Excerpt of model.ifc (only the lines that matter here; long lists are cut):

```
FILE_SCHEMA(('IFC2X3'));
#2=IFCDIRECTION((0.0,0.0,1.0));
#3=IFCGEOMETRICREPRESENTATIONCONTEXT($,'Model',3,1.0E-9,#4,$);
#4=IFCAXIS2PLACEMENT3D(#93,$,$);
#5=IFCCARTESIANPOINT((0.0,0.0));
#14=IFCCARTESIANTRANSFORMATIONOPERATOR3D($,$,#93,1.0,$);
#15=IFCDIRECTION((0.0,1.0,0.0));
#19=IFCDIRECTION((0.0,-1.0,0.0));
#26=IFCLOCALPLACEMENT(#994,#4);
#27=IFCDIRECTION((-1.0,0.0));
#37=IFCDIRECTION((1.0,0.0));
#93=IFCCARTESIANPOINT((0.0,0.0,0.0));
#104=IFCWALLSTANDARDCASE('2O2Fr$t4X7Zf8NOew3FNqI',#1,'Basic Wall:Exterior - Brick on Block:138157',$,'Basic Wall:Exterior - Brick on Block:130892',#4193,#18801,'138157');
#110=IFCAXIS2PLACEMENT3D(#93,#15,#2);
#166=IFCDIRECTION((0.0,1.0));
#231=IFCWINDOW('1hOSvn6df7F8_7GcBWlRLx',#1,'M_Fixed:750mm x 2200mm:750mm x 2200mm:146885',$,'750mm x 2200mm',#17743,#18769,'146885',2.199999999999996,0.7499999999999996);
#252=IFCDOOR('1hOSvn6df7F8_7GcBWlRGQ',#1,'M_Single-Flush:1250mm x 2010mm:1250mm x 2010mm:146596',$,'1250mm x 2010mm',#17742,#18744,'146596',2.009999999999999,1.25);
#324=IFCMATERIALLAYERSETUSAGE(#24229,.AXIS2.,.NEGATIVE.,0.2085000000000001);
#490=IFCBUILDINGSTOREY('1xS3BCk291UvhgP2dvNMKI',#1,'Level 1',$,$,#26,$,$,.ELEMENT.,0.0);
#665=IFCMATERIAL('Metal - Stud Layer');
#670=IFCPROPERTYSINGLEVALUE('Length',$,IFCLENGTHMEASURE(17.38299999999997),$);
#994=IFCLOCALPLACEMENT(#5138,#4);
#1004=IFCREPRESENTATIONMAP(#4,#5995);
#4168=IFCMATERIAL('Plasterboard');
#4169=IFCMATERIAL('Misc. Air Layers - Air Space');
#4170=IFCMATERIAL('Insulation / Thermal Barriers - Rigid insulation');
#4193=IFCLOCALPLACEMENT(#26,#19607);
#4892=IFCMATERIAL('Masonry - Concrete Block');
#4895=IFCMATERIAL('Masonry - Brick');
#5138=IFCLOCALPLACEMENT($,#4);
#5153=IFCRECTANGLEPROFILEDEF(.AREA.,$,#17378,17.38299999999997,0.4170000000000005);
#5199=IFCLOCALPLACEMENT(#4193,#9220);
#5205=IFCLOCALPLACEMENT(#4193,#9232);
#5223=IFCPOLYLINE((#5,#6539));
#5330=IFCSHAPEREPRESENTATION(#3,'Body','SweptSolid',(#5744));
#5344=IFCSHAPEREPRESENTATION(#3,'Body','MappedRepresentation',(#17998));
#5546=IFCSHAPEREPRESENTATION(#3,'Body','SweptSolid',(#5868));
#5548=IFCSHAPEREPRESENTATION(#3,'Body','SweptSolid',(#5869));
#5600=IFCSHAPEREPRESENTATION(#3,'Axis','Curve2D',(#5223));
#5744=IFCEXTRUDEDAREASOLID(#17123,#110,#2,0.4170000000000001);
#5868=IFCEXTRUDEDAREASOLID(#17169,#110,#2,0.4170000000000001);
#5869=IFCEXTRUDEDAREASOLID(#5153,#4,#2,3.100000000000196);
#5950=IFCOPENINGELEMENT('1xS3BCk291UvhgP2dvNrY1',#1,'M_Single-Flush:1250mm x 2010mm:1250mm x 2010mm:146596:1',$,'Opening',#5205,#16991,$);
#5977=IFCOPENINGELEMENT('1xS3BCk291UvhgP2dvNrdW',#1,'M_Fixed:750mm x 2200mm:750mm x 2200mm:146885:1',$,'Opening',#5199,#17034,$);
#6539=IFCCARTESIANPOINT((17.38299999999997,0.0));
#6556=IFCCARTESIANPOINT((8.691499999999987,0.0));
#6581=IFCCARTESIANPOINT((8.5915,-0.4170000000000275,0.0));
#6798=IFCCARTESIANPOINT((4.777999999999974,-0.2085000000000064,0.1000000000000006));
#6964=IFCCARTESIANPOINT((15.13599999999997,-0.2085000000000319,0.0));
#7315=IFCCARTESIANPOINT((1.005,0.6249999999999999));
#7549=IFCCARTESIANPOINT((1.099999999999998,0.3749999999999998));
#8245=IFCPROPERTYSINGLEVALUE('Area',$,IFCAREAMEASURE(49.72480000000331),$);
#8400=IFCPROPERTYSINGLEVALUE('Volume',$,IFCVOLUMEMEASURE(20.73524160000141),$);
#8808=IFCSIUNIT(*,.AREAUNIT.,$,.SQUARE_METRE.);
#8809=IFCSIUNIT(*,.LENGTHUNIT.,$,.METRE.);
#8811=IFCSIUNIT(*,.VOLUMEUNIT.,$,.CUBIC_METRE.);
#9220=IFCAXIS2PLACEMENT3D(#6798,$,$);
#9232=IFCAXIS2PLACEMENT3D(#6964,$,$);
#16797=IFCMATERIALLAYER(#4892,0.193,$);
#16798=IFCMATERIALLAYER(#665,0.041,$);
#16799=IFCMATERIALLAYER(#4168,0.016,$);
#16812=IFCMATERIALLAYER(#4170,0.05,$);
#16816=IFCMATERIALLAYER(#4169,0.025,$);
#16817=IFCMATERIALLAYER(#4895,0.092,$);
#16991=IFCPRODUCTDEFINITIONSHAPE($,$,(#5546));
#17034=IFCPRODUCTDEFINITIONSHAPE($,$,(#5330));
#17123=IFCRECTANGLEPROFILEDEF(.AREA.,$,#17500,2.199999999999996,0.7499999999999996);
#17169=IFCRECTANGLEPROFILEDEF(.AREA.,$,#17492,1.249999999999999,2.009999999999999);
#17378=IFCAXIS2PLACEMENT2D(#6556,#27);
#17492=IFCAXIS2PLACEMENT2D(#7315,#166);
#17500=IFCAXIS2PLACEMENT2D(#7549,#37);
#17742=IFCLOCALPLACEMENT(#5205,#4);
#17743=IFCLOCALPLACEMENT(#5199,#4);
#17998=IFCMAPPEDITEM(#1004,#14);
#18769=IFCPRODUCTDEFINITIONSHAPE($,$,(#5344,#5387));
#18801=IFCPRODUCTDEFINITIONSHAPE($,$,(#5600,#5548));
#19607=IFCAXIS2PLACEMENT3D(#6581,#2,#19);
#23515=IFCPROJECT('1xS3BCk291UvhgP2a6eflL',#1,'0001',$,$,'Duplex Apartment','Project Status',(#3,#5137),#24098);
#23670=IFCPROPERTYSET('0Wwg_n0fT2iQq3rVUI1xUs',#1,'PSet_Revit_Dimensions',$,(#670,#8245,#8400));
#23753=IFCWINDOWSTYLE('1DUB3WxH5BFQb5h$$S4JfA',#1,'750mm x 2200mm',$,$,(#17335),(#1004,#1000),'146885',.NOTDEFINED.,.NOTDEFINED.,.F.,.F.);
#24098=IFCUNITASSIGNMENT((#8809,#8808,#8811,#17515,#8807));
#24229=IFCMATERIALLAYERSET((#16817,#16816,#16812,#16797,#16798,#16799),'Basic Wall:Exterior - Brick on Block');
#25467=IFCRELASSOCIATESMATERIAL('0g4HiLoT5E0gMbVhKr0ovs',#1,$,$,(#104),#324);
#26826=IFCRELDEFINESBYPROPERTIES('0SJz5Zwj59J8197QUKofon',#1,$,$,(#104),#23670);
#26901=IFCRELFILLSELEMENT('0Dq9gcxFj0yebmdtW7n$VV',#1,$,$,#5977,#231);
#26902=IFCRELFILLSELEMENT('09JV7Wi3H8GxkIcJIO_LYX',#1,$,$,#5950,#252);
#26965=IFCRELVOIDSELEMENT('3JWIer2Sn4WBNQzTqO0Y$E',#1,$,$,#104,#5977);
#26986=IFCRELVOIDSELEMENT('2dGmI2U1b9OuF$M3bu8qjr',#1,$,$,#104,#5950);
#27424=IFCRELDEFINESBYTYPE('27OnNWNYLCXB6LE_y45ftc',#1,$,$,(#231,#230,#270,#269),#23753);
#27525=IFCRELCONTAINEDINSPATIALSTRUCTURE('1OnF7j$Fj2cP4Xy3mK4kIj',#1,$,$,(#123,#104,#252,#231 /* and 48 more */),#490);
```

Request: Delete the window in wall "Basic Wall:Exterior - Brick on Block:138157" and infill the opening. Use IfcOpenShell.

```python
import ifcopenshell
import ifcopenshell.api.feature
import ifcopenshell.api.pset
import ifcopenshell.api.root
import ifcopenshell.geom
import ifcopenshell.util.element
import ifcopenshell.util.shape
import ifcopenshell.util.unit

model = ifcopenshell.open("model.ifc")
area_scale = ifcopenshell.util.unit.calculate_unit_scale(model, "AREAUNIT")
volume_scale = ifcopenshell.util.unit.calculate_unit_scale(model, "VOLUMEUNIT")
settings = ifcopenshell.geom.settings()


def volume(element):
    """Net volume in cubic metres, openings subtracted."""
    shape = ifcopenshell.geom.create_shape(settings, element)
    return ifcopenshell.util.shape.get_volume(shape.geometry)


window = model.by_guid("1hOSvn6df7F8_7GcBWlRLx")
opening = window.FillsVoids[0].RelatingOpeningElement
wall = opening.VoidsElements[0].RelatingBuildingElement
before = volume(wall)

ifcopenshell.api.root.remove_product(model, product=window)
ifcopenshell.api.feature.remove_feature(model, feature=opening)

after = volume(wall)
thickness = 0.417  # wall thickness in metres

# Update the wall's stored quantities.
pset = model.by_id(ifcopenshell.util.element.get_pset(wall, "PSet_Revit_Dimensions", should_inherit=False)["id"])
ifcopenshell.api.pset.edit_pset(model, pset=pset, properties={
    "Area": model.create_entity("IfcAreaMeasure", after / thickness / area_scale),
    "Volume": model.create_entity("IfcVolumeMeasure", after / volume_scale),
})

print(f"wall volume {before:.3f} -> {after:.3f} m3")

model.write("model-out.ifc")
```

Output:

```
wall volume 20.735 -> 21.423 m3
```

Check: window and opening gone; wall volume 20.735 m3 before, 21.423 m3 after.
